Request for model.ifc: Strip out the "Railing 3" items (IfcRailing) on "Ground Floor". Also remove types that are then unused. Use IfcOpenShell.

First a look at what the model holds.

```python
import ifcopenshell
import ifcopenshell.util.element

model = ifcopenshell.open("model.ifc")
print(model.schema)
storey = next(s for s in model.by_type("IfcBuildingStorey") if s.Name == "Ground Floor")
railings = [e for e in ifcopenshell.util.element.get_decomposition(storey) if e.is_a("IfcRailing")]
seen = {}
for e in railings:
    element_type = ifcopenshell.util.element.get_type(e)
    name = element_type.Name if element_type not in (None, e) else None
    seen[name] = seen.get(name, 0) + 1
for name, count in sorted(seen.items(), key=str):
    print(count, "x", name)
```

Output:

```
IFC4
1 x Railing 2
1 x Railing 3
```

```python
import ifcopenshell
import ifcopenshell.api.root
import ifcopenshell.util.element

model = ifcopenshell.open("model.ifc")

storey = next(s for s in model.by_type("IfcBuildingStorey") if s.Name == "Ground Floor")
railings = [e for e in ifcopenshell.util.element.get_decomposition(storey) if e.is_a("IfcRailing")]
targets = [e for e in railings if (t := ifcopenshell.util.element.get_type(e)) not in (None, e) and t.Name == "Railing 3"]
types = {ifcopenshell.util.element.get_type(e) for e in targets} - {None, *targets}

for e in targets:
    ifcopenshell.api.root.remove_product(model, product=e)
print(len(targets), "removed")

unused = [t for t in types if not ifcopenshell.util.element.get_types(t)]
for t in unused:
    ifcopenshell.api.root.remove_product(model, product=t)
print(len(unused), "unused types removed")

model.write("model_edited.ifc")
```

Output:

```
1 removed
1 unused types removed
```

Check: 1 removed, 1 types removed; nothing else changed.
